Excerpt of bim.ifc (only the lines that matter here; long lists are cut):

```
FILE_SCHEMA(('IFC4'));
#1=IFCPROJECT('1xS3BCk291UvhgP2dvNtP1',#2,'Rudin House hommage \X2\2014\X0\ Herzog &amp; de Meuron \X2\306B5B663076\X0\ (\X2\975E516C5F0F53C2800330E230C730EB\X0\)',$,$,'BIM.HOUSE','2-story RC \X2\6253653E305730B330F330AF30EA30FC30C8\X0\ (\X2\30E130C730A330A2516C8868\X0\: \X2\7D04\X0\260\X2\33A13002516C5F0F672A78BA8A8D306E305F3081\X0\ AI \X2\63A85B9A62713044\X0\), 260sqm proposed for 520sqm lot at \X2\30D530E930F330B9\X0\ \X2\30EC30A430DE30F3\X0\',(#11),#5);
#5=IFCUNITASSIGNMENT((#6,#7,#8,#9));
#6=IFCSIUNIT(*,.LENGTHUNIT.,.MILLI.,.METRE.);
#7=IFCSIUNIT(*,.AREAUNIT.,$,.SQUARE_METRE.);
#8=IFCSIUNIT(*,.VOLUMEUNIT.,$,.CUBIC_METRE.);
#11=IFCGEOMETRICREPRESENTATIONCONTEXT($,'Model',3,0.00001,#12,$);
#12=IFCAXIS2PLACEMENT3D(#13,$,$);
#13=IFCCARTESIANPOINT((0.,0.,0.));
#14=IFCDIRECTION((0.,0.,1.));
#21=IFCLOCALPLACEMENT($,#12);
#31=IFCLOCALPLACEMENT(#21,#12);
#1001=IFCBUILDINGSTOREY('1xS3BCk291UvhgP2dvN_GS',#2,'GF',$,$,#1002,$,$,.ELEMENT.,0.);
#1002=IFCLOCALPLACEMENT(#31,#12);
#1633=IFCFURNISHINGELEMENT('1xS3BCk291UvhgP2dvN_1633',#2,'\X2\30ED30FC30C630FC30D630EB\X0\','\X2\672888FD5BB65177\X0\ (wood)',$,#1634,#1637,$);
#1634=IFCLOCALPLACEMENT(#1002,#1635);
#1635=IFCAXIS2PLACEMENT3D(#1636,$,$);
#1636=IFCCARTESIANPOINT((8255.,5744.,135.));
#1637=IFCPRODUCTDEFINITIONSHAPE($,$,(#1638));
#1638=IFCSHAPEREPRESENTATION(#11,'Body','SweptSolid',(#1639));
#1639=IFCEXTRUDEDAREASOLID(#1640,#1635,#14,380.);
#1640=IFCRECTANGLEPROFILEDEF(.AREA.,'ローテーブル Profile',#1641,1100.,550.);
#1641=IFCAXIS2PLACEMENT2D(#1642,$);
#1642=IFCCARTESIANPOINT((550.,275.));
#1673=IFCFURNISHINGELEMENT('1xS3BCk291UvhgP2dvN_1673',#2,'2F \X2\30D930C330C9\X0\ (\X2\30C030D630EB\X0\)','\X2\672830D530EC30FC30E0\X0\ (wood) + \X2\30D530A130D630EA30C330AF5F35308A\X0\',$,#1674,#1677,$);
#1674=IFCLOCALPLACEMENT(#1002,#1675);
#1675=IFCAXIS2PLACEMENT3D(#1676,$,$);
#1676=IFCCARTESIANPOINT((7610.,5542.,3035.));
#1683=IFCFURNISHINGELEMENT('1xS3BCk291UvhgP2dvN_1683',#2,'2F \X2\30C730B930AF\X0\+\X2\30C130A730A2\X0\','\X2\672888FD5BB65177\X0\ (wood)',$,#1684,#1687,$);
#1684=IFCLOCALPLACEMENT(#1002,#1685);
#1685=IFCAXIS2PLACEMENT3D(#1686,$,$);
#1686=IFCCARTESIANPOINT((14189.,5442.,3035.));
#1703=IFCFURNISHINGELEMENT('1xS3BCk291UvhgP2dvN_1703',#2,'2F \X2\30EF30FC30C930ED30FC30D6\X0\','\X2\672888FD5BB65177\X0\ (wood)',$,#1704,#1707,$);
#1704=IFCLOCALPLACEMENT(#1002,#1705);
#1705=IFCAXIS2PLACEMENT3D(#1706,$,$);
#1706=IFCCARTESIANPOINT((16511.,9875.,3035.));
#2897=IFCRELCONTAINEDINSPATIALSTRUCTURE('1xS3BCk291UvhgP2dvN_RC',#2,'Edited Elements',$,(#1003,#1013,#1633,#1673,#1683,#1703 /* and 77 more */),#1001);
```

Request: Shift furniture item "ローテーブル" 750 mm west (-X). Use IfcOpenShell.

```python
import ifcopenshell
import ifcopenshell.api.geometry
import ifcopenshell.util.placement
import ifcopenshell.util.unit

model = ifcopenshell.open("bim.ifc")
unit_scale = ifcopenshell.util.unit.calculate_unit_scale(model)

item = model.by_id(1633)
matrix = ifcopenshell.util.placement.get_local_placement(item.ObjectPlacement)
matrix[0, 3] -= 0.75 / unit_scale
ifcopenshell.api.geometry.edit_object_placement(model, product=item, matrix=matrix, is_si=False)

print(ifcopenshell.util.placement.get_local_placement(item.ObjectPlacement).round(3) + 0.0)

model.write("bim_updated.ifc")
```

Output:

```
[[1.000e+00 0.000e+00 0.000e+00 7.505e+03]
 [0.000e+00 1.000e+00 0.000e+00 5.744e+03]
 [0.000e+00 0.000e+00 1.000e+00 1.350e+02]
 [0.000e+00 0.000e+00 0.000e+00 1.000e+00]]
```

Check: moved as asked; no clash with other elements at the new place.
